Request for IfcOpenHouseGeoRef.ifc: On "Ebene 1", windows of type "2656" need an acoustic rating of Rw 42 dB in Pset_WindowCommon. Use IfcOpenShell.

First a look at what the model holds.

```python
import ifcopenshell
import ifcopenshell.util.element

model = ifcopenshell.open("IfcOpenHouseGeoRef.ifc")
print(model.schema)
storey = next(s for s in model.by_type("IfcBuildingStorey") if s.Name == "Ebene 1")
windows = [e for e in ifcopenshell.util.element.get_decomposition(storey) if e.is_a("IfcWindow")]
seen = {}
for e in windows:
    element_type = ifcopenshell.util.element.get_type(e)
    key = (element_type.Name if element_type != e and element_type else None, ifcopenshell.util.element.get_pset(e, "Pset_WindowCommon", "AcousticRating"))
    seen[key] = seen.get(key, 0) + 1
for (name, value), count in sorted(seen.items(), key=str):
    print(count, "x", name, "|", value)
```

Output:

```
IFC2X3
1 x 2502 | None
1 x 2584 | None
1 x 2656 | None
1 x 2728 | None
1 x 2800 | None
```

```python
import ifcopenshell
import ifcopenshell.api.pset
import ifcopenshell.util.element

model = ifcopenshell.open("IfcOpenHouseGeoRef.ifc")

storey = next(s for s in model.by_type("IfcBuildingStorey") if s.Name == "Ebene 1")
windows = [e for e in ifcopenshell.util.element.get_decomposition(storey) if e.is_a("IfcWindow")]

count = 0
for e in windows:
    element_type = ifcopenshell.util.element.get_type(e)
    if element_type in (None, e) or element_type.Name != "2656":
        continue
    # add_pset returns the element's existing set when there is one.
    pset = ifcopenshell.api.pset.add_pset(model, product=e, name="Pset_WindowCommon")
    ifcopenshell.api.pset.edit_pset(model, pset=pset, properties={"AcousticRating": "Rw 42 dB"})
    count += 1

print(count, "windows updated")

model.write("IfcOpenHouseGeoRef-out.ifc")
```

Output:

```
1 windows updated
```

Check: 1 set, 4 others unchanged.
